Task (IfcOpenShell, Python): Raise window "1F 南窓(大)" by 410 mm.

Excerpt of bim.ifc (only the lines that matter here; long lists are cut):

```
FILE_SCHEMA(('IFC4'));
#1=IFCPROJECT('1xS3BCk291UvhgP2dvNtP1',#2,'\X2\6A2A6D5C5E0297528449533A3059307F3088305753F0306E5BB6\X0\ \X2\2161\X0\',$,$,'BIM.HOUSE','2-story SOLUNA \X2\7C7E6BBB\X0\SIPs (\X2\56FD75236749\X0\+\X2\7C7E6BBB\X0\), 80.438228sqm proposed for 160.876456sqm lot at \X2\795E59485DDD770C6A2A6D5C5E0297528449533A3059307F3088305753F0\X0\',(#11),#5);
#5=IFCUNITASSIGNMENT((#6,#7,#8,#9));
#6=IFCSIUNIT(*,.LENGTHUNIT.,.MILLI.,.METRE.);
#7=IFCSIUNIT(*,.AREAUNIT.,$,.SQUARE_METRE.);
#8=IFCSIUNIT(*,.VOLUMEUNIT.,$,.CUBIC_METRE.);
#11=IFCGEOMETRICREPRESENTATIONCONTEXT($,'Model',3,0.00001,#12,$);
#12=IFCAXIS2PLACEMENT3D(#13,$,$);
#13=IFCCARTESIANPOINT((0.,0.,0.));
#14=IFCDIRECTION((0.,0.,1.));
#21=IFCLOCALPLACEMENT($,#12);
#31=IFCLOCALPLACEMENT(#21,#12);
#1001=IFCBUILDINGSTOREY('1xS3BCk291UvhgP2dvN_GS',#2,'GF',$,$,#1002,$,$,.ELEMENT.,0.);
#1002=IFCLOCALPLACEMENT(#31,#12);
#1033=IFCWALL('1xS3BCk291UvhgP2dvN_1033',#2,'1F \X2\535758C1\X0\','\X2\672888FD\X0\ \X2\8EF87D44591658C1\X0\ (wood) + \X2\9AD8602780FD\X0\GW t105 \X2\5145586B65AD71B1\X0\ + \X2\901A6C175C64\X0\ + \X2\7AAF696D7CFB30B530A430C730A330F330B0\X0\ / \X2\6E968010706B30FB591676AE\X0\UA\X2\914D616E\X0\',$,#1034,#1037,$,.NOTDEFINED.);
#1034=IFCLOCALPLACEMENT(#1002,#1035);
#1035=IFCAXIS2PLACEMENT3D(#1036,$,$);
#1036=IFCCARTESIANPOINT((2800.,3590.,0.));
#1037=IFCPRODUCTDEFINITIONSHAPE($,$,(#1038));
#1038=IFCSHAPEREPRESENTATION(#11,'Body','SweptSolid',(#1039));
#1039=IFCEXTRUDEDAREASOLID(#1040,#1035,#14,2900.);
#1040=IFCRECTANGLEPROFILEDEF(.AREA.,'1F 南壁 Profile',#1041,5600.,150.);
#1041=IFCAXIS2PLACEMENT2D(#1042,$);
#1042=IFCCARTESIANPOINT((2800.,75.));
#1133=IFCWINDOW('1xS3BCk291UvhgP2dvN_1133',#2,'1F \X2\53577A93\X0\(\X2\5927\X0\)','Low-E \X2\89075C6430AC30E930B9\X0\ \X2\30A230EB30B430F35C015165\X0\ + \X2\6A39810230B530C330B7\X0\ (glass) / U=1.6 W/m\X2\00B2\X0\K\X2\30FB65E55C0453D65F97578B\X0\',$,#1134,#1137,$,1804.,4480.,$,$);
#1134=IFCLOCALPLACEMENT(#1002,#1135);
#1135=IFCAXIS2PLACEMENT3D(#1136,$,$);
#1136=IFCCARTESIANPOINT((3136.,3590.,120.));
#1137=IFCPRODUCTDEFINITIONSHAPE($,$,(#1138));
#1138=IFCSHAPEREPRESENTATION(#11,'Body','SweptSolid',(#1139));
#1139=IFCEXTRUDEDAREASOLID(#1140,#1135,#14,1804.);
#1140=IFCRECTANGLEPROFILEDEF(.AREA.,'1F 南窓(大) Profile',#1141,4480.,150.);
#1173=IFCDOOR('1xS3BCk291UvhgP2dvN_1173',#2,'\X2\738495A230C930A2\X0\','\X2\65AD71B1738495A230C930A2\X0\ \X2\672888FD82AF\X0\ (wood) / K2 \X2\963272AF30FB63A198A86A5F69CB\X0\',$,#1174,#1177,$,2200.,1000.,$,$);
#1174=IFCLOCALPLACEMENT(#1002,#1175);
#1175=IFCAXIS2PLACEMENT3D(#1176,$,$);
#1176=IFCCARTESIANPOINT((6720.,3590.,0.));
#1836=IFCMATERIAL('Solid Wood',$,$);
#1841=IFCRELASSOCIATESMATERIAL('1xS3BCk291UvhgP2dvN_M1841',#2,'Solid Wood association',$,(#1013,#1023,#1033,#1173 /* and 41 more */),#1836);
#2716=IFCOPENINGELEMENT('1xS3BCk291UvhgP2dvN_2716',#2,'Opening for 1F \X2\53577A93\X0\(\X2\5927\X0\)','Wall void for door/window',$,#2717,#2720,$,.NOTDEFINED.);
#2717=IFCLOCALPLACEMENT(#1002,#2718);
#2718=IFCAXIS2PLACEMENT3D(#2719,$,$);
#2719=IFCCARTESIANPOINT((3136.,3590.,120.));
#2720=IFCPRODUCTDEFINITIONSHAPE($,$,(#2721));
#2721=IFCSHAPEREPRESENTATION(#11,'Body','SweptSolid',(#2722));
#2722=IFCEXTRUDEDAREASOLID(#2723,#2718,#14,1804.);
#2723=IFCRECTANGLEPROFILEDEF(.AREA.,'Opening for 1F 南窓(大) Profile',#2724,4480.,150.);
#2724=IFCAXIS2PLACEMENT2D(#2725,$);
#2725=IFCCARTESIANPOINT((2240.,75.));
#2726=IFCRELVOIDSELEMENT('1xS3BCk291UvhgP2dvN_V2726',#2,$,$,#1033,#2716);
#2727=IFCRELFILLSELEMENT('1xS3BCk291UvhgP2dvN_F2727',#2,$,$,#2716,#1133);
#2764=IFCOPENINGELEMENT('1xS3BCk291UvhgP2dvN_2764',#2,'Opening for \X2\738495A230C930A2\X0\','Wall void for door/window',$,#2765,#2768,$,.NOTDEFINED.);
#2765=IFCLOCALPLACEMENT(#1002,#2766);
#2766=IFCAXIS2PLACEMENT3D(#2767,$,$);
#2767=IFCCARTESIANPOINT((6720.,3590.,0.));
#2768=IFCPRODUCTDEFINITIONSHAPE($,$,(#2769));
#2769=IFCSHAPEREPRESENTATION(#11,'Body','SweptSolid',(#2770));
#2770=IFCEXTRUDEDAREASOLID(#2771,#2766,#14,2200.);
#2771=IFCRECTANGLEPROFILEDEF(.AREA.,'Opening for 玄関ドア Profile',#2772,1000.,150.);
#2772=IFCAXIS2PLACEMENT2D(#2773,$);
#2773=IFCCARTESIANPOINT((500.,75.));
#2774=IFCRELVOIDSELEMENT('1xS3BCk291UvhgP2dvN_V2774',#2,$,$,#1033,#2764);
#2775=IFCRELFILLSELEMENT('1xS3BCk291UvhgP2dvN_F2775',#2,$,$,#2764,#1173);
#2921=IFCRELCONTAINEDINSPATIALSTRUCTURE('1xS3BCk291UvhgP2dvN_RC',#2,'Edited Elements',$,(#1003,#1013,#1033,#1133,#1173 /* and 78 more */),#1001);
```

```python
import numpy as np
import ifcopenshell
import ifcopenshell.api.geometry
import ifcopenshell.util.placement
import ifcopenshell.util.unit

model = ifcopenshell.open("bim.ifc")
unit_scale = ifcopenshell.util.unit.calculate_unit_scale(model)

window = model.by_guid("1xS3BCk291UvhgP2dvN_1133")
opening = window.FillsVoids[0].RelatingOpeningElement
dz = 410.0

shift = np.array([0.0, 0.0, dz])
# The window is not placed relative to its opening, so move both.
for product in (opening, window):
    matrix = ifcopenshell.util.placement.get_local_placement(product.ObjectPlacement)
    matrix[:3, 3] += shift
    ifcopenshell.api.geometry.edit_object_placement(model, product=product, matrix=matrix, is_si=False)

print(f"moved by {dz * unit_scale:+.3f} m")

model.write("bim_updated.ifc")
```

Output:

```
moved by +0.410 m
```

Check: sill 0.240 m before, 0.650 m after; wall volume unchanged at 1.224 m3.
